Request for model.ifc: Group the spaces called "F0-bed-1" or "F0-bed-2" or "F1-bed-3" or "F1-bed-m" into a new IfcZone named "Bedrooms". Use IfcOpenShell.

First a look at what the model holds.

```python
import ifcopenshell

model = ifcopenshell.open("model.ifc")
print(model.schema)
seen = {}
for space in model.by_type("IfcSpace"):
    seen[space.LongName] = seen.get(space.LongName, 0) + 1
for name, count in sorted(seen.items(), key=str):
    print(count, "x", name)
print("zones:", [z.Name for z in model.by_type("IfcZone")][:20])
```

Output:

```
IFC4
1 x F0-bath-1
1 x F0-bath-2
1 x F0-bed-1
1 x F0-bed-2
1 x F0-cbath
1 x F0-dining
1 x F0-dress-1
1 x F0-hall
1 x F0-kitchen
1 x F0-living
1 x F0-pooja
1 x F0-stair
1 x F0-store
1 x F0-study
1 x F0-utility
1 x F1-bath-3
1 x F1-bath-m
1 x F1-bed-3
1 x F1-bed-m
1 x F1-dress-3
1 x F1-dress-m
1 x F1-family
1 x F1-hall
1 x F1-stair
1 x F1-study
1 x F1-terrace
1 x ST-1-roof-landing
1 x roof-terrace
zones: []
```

```python
import ifcopenshell
import ifcopenshell.api.group
import ifcopenshell.api.root

model = ifcopenshell.open("model.ifc")

names = {"F0-bed-1", "F0-bed-2", "F1-bed-3", "F1-bed-m"}
spaces = [s for s in model.by_type("IfcSpace") if s.LongName in names]

zone = ifcopenshell.api.root.create_entity(model, ifc_class="IfcZone", name="Bedrooms")
ifcopenshell.api.group.assign_group(model, products=spaces, group=zone)
print(len(spaces), "spaces in", zone.Name)

model.write("model_v2.ifc")
```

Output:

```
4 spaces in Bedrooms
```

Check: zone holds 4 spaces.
